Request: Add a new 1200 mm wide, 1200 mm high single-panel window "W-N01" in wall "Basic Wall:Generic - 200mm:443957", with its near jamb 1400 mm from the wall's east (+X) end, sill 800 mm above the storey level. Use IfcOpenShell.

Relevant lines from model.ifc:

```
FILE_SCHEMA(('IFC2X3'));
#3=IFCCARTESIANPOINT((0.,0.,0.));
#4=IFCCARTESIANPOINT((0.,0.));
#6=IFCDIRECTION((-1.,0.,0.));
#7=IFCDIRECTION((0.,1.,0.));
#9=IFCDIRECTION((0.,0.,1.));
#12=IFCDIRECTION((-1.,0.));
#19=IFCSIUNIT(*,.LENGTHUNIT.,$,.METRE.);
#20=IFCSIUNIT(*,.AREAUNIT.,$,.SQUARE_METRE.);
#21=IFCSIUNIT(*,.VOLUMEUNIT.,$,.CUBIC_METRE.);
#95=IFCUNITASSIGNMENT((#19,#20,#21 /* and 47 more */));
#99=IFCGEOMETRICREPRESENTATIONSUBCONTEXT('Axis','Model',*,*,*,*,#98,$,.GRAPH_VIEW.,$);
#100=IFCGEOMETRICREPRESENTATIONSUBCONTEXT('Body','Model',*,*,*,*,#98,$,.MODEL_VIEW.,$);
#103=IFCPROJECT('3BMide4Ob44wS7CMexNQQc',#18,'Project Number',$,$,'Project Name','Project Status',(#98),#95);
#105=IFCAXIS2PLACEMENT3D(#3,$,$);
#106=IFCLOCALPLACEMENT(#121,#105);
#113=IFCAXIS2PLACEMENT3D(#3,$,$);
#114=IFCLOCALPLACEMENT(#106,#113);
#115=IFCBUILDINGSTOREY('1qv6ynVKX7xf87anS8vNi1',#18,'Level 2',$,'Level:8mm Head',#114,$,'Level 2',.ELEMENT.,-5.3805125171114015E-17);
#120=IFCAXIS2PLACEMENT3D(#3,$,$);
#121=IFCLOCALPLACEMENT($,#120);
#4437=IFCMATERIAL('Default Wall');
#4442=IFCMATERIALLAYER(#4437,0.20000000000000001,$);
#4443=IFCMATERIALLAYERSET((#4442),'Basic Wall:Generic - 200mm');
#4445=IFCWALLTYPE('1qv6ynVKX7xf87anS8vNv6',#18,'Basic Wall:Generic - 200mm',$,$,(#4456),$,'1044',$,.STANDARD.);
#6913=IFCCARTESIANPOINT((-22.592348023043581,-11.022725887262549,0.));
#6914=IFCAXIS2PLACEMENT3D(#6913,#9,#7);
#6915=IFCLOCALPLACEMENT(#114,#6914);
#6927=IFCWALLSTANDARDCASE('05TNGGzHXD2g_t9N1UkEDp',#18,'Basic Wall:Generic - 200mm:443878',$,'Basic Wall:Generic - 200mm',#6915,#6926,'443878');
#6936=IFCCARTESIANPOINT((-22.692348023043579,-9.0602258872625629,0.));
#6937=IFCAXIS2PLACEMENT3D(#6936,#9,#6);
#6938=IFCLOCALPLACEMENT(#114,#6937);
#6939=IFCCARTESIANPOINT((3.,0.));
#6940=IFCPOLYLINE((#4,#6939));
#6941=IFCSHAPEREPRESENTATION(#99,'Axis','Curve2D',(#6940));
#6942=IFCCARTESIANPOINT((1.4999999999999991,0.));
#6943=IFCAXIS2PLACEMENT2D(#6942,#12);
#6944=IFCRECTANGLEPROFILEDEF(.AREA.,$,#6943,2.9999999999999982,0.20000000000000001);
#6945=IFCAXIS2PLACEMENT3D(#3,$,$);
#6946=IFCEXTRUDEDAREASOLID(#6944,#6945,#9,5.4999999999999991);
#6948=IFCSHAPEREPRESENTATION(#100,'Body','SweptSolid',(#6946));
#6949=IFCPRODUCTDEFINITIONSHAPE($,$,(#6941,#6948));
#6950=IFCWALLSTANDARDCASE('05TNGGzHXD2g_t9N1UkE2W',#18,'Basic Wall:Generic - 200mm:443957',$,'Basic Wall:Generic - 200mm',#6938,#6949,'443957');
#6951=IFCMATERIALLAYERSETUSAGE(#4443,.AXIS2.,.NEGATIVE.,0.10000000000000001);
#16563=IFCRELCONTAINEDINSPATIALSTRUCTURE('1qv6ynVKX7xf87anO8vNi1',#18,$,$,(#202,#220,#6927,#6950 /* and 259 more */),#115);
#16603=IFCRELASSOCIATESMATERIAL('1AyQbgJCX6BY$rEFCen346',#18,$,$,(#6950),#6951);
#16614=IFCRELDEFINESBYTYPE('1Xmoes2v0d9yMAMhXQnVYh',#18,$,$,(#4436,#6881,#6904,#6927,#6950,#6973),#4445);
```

```python
import numpy as np
import ifcopenshell
import ifcopenshell.api.feature
import ifcopenshell.api.geometry
import ifcopenshell.api.root
import ifcopenshell.api.spatial
import ifcopenshell.api.type
import ifcopenshell.geom
import ifcopenshell.util.element
import ifcopenshell.util.placement
import ifcopenshell.util.representation
import ifcopenshell.util.shape
import ifcopenshell.util.unit

model = ifcopenshell.open("model.ifc")
unit_scale = ifcopenshell.util.unit.calculate_unit_scale(model)
settings = ifcopenshell.geom.settings()


def volume(element):
    """Net volume in cubic metres, openings subtracted."""
    shape = ifcopenshell.geom.create_shape(settings, element)
    return ifcopenshell.util.shape.get_volume(shape.geometry)


wall = model.by_id(6950)
storey = ifcopenshell.util.element.get_container(wall, ifc_class="IfcBuildingStorey")
context = ifcopenshell.util.representation.get_context(model, "Model", "Body", "MODEL_VIEW")
before = volume(wall)

width, height, from_end, sill = 1.2, 1.2, 1.4, 0.8  # metres

# The wall runs along its own X axis, and the end named is its -X end.
wall_shape = ifcopenshell.geom.create_shape(settings, wall)
x, y, z = ifcopenshell.util.shape.get_vertices(wall_shape.geometry).T
start = x.min() + from_end
face, thickness = float(y.min()), float(y.max() - y.min())
wall_matrix = ifcopenshell.util.placement.get_local_placement(wall.ObjectPlacement)
level = ifcopenshell.util.placement.get_local_placement(storey.ObjectPlacement)[2, 3]


def in_wall(x, y):
    """Placement at x, y metres in the wall's axes, at sill height."""
    matrix = wall_matrix.copy()
    matrix[:, 3] = wall_matrix @ np.array([x / unit_scale, y / unit_scale, 0.0, 1.0])
    matrix[2, 3] = level + sill / unit_scale
    return matrix


# Opening: a box that overshoots both wall faces by 50 mm.
opening = ifcopenshell.api.root.create_entity(model, ifc_class="IfcOpeningElement")
box = ifcopenshell.api.geometry.add_wall_representation(
    model, context=context, length=width, height=height, thickness=thickness + 0.1
)
ifcopenshell.api.geometry.assign_representation(model, product=opening, representation=box)
ifcopenshell.api.geometry.edit_object_placement(model, product=opening, matrix=in_wall(start, face - 0.05), is_si=False)
ifcopenshell.api.feature.add_feature(model, feature=opening, element=wall)

window = ifcopenshell.api.root.create_entity(model, ifc_class="IfcWindow", name="W-N01")
window.OverallWidth, window.OverallHeight = width / unit_scale, height / unit_scale
body = ifcopenshell.api.geometry.add_window_representation(
    model,
    context=context,
    overall_width=window.OverallWidth,
    overall_height=window.OverallHeight,
    partition_type="SINGLE_PANEL",
)
ifcopenshell.api.geometry.assign_representation(model, product=window, representation=body)
ifcopenshell.api.spatial.assign_container(model, products=[window], relating_structure=storey)
fills = ifcopenshell.api.feature.add_filling(model, opening=opening, element=window)
fills.OwnerHistory = window.OwnerHistory  # required in IFC2X3

# IFC2X3 keeps the operation on the window style.
style = ifcopenshell.api.root.create_entity(model, ifc_class="IfcWindowStyle", name="W-N01")
style.OperationType, style.ConstructionType = "SINGLE_PANEL", "NOTDEFINED"
style.ParameterTakesPrecedence = style.Sizeable = False
ifcopenshell.api.type.assign_type(model, related_objects=[window], relating_type=style)

# Centre the window in the wall's thickness.
ifcopenshell.api.geometry.edit_object_placement(model, product=window, matrix=in_wall(start, face), is_si=False)
window_shape = ifcopenshell.geom.create_shape(settings, window)
depth = ifcopenshell.util.shape.get_vertices(window_shape.geometry)[:, 1]
offset = face + thickness / 2 - (depth.min() + depth.max()) / 2
ifcopenshell.api.geometry.edit_object_placement(model, product=window, matrix=in_wall(start, offset), is_si=False)

after = volume(wall)

print(f"wall volume {before:.3f} -> {after:.3f} m3")

model.write("model_edited.ifc")
```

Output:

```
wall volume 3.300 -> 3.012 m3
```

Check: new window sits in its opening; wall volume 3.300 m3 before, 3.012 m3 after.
